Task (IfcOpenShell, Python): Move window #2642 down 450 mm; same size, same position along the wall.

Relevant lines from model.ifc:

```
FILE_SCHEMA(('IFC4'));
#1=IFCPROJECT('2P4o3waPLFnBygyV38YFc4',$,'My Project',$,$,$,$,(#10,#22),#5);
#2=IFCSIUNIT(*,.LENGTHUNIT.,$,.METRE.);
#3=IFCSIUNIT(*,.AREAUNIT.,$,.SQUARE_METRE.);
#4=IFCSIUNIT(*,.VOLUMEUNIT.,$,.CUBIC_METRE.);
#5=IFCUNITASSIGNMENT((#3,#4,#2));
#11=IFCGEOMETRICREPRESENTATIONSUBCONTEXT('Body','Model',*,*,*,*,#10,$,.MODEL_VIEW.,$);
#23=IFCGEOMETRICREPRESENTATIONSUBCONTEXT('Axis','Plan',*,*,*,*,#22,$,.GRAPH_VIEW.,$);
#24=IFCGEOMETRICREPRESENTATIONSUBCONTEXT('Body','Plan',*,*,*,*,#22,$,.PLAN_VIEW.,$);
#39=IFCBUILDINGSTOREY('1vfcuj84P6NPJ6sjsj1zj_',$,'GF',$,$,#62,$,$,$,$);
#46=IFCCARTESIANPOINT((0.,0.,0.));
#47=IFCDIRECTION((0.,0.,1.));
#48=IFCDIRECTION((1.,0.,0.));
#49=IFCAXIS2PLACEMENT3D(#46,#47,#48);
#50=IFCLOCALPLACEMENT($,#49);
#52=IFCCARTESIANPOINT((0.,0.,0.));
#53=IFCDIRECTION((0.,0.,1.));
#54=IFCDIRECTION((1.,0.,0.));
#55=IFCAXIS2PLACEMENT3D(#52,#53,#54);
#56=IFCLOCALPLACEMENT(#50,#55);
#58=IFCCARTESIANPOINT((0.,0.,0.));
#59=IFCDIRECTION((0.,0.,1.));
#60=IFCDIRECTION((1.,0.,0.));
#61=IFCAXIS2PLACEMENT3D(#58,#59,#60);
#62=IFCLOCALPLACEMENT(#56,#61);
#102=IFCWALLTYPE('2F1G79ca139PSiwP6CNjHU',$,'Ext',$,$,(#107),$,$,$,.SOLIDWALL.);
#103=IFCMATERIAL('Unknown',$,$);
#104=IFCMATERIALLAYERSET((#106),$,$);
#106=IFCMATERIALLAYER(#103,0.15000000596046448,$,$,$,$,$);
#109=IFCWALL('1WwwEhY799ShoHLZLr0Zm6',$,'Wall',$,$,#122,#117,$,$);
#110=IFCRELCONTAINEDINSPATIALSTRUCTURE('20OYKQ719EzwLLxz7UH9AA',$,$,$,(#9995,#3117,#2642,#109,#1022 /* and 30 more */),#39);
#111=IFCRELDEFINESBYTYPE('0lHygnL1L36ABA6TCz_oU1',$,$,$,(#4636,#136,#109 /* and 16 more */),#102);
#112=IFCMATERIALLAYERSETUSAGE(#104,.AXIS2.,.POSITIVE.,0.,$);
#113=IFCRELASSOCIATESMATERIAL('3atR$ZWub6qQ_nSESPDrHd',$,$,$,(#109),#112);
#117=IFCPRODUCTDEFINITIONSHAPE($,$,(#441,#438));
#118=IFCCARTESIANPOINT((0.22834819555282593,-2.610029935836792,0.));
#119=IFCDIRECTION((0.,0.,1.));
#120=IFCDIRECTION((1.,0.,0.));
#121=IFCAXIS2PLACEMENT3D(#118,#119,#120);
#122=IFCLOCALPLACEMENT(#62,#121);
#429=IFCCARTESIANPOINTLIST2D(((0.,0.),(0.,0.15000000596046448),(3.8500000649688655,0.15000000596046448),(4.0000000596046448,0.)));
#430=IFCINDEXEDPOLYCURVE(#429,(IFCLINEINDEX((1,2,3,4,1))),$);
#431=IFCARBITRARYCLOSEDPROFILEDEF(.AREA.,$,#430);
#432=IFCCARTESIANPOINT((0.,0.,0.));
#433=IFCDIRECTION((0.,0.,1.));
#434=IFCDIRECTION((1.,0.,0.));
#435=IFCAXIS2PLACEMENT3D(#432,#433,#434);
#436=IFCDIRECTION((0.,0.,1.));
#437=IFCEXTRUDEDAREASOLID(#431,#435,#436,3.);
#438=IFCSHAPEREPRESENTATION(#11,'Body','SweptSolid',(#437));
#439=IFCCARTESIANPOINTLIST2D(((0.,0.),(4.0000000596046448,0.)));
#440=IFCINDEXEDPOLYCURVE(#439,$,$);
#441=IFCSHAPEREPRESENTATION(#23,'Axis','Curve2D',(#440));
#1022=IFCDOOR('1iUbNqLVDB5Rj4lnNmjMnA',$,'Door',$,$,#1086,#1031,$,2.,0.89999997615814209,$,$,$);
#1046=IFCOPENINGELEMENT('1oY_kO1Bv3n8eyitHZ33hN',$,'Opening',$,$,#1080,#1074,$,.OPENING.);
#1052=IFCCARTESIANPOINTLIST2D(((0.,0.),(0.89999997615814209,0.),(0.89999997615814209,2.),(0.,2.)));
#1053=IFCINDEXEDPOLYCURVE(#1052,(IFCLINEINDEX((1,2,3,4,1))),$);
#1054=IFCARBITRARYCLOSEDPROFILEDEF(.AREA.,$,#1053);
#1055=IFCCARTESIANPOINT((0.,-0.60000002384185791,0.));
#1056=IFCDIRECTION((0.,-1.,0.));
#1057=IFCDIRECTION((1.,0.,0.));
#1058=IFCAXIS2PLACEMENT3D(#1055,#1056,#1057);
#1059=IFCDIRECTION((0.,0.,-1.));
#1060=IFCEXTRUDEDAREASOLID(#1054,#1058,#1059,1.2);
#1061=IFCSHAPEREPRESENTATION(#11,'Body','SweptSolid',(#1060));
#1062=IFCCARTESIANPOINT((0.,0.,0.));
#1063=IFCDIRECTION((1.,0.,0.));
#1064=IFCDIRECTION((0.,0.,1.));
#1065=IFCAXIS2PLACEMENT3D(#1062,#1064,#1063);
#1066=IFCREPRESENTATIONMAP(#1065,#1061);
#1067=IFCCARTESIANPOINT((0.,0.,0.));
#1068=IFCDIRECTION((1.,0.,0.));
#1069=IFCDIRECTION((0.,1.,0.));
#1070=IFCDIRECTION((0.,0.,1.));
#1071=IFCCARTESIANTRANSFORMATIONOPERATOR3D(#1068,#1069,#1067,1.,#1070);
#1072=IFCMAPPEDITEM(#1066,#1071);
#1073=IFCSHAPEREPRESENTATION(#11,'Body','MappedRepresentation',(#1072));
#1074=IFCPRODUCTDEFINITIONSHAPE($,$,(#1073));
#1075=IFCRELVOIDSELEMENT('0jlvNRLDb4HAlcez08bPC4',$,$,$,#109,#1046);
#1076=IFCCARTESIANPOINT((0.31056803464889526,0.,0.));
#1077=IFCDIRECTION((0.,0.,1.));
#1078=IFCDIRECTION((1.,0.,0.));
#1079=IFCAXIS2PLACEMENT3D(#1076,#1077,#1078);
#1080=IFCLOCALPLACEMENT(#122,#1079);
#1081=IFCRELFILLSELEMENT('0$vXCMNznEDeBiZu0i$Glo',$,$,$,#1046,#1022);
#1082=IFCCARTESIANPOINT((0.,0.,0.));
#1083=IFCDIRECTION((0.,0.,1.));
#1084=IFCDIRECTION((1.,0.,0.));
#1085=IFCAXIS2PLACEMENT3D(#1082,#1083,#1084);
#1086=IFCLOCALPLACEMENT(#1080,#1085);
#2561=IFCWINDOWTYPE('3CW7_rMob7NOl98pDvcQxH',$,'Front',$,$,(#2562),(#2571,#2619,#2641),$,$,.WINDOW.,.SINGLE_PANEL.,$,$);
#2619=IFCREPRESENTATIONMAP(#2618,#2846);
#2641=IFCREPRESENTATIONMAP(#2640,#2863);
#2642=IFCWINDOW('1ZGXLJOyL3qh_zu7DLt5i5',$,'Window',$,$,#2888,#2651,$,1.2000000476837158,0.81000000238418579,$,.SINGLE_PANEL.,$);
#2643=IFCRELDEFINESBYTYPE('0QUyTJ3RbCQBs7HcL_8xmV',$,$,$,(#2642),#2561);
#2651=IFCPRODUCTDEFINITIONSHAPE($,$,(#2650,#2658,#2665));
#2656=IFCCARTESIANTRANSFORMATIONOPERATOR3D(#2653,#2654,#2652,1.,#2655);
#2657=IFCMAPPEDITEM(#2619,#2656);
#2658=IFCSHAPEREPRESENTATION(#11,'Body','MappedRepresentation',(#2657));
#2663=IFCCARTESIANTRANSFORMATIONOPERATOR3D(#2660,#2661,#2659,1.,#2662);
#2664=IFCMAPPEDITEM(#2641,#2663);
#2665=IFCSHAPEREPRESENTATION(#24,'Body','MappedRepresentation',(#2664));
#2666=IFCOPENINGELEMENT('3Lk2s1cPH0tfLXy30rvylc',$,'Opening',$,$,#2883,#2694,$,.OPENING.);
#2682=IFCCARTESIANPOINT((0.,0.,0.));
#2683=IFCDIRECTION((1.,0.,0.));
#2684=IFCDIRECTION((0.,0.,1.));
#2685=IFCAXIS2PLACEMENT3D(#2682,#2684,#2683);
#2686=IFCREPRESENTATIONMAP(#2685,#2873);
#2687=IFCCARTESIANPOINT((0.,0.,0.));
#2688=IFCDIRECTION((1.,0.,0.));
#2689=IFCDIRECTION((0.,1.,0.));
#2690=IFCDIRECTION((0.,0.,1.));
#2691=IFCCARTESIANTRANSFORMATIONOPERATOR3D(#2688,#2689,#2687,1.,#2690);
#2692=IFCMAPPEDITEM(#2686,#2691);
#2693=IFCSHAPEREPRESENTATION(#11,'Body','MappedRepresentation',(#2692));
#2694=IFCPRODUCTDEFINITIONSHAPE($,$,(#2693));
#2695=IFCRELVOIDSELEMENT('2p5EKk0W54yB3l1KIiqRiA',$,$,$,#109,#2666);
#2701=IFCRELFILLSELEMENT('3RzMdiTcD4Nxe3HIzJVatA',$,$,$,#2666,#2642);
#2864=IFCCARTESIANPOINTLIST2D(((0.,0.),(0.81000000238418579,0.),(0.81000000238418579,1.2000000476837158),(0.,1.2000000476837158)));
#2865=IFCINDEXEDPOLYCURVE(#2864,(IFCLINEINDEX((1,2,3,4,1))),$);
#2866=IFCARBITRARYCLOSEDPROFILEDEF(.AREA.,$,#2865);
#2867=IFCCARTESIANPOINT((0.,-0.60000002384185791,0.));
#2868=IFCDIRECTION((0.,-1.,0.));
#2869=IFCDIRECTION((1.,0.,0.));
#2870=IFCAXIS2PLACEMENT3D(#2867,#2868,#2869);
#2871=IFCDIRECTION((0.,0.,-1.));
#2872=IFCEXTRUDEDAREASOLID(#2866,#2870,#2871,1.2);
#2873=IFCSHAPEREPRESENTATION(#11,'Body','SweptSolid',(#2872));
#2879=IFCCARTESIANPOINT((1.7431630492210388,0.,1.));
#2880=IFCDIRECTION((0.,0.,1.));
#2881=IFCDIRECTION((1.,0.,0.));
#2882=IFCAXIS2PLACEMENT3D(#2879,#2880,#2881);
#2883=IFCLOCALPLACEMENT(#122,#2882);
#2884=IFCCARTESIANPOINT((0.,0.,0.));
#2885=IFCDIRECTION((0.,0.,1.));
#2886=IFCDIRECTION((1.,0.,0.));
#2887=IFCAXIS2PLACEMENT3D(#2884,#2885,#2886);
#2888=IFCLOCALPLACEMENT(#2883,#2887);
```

```python
import numpy as np
import ifcopenshell
import ifcopenshell.api.geometry
import ifcopenshell.util.placement
import ifcopenshell.util.unit

model = ifcopenshell.open("model.ifc")
unit_scale = ifcopenshell.util.unit.calculate_unit_scale(model)

window = model.by_id(2642)
opening = window.FillsVoids[0].RelatingOpeningElement
dz = -0.45 / unit_scale

shift = np.array([0.0, 0.0, dz])
# The window is placed relative to its opening, so it follows when the opening moves.
matrix = ifcopenshell.util.placement.get_local_placement(opening.ObjectPlacement)
matrix[:3, 3] += shift
ifcopenshell.api.geometry.edit_object_placement(
    model, product=opening, matrix=matrix, is_si=False, should_transform_children=True
)

print(f"moved by {dz * unit_scale:+.3f} m")

model.write("model_edited.ifc")
```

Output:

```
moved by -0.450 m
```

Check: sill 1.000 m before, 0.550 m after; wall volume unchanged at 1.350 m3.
